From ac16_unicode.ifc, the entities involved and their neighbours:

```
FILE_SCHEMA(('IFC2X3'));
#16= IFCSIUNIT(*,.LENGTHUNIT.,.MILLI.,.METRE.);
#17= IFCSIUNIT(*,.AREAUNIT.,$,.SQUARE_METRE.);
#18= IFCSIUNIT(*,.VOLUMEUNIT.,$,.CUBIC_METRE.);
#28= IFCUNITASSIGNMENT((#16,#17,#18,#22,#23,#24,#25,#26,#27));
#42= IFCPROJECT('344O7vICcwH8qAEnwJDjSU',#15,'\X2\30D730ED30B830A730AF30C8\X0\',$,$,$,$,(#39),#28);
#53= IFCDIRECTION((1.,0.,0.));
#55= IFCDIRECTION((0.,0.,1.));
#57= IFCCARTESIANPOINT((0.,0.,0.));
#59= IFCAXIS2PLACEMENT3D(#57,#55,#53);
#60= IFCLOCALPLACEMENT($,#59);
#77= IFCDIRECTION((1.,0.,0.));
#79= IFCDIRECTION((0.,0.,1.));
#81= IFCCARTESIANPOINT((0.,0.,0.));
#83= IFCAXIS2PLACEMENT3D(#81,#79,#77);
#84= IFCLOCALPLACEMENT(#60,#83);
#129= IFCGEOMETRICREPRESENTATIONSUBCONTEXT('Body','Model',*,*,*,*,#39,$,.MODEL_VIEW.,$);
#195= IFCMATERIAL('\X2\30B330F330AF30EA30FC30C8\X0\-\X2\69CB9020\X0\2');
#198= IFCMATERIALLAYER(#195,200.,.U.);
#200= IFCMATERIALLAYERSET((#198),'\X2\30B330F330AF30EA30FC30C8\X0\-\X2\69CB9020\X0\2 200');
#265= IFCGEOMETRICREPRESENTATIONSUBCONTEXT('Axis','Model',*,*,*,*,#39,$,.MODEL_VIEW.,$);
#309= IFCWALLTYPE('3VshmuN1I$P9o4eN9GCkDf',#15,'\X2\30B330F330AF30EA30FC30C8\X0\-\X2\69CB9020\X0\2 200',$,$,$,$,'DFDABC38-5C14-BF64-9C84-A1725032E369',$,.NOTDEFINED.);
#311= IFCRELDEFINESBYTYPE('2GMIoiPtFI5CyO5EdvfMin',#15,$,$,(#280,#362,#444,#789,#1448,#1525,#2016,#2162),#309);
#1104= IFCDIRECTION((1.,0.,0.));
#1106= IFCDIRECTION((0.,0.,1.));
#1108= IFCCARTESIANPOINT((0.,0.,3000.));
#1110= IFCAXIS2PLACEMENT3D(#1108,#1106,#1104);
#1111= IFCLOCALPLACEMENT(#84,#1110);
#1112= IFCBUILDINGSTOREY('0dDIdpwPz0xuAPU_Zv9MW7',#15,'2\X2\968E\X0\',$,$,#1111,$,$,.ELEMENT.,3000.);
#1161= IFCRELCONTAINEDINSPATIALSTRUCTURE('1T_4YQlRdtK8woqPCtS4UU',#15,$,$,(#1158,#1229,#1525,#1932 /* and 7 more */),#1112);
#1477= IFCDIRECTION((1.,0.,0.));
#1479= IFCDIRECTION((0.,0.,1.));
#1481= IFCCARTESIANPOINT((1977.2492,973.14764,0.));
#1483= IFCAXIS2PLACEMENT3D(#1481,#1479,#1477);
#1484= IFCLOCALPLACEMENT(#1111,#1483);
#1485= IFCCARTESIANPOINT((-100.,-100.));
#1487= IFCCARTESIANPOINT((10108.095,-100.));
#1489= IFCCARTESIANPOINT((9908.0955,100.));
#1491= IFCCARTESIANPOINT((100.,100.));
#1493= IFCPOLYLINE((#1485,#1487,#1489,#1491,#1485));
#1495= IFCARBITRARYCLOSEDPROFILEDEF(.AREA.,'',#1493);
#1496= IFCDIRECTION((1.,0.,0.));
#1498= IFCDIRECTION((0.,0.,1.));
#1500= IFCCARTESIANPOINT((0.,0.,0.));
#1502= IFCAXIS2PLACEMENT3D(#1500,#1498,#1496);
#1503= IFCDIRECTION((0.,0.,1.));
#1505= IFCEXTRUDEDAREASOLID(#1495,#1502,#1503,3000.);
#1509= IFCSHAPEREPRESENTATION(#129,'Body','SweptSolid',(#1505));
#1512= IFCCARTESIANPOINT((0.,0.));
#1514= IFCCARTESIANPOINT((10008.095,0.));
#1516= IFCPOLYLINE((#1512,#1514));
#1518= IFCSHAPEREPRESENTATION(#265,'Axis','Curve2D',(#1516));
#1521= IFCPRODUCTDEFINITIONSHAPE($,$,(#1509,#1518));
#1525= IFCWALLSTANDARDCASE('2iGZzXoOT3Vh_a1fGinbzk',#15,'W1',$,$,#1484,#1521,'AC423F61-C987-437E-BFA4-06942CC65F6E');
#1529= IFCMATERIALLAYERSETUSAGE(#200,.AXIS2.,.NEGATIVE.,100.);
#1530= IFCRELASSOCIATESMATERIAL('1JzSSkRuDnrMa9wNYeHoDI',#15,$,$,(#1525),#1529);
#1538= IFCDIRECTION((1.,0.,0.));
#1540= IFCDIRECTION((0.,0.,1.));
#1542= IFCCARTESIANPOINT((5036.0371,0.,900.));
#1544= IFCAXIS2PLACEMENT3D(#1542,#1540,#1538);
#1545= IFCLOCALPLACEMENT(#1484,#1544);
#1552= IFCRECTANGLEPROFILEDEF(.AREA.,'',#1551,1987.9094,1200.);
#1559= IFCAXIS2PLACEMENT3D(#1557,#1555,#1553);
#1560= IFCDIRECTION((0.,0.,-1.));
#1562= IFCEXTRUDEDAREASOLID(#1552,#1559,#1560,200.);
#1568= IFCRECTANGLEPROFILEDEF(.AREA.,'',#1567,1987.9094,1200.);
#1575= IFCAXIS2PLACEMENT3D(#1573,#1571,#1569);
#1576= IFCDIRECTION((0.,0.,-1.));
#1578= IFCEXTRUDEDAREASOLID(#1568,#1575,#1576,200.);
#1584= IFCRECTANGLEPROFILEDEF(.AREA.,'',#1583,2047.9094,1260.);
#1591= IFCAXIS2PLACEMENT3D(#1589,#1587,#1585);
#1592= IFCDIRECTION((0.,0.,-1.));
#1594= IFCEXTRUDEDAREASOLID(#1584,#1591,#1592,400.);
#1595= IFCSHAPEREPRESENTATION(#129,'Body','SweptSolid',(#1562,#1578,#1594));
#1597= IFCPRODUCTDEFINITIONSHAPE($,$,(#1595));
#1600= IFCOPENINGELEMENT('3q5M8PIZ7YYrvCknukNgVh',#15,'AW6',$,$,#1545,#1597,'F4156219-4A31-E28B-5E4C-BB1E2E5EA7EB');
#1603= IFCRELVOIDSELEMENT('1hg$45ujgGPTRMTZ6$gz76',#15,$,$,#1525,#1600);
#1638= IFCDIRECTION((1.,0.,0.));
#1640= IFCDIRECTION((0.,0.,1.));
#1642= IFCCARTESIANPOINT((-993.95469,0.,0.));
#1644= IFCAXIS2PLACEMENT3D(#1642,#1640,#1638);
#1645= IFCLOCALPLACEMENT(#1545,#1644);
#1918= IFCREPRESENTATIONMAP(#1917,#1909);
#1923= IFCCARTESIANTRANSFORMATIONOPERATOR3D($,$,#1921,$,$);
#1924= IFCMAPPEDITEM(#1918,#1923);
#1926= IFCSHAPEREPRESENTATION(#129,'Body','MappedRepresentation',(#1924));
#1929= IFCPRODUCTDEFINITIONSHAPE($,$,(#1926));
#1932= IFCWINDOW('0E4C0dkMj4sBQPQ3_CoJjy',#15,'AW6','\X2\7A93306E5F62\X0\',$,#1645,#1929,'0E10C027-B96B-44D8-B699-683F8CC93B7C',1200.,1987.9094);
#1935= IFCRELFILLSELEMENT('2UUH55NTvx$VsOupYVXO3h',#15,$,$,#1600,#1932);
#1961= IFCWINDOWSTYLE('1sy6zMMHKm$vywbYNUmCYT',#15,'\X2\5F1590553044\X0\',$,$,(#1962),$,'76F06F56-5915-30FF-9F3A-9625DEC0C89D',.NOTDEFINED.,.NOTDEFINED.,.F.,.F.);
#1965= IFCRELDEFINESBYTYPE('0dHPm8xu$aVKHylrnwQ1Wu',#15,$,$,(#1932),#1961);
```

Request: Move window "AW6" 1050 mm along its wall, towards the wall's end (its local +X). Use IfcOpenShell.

```python
import ifcopenshell
import ifcopenshell.api.geometry
import ifcopenshell.util.placement

model = ifcopenshell.open("ac16_unicode.ifc")

window = model.by_guid("0E4C0dkMj4sBQPQ3_CoJjy")
opening = window.FillsVoids[0].RelatingOpeningElement
wall = opening.VoidsElements[0].RelatingBuildingElement

wall_matrix = ifcopenshell.util.placement.get_local_placement(wall.ObjectPlacement)
shift = wall_matrix[:3, 0] * 1050.0
before = ifcopenshell.util.placement.get_local_placement(window.ObjectPlacement)[:3, 3].copy()

# The window is placed relative to its opening, so it follows when the opening moves.
matrix = ifcopenshell.util.placement.get_local_placement(opening.ObjectPlacement)
matrix[:3, 3] += shift
ifcopenshell.api.geometry.edit_object_placement(
    model, product=opening, matrix=matrix, is_si=False, should_transform_children=True
)

after = ifcopenshell.util.placement.get_local_placement(window.ObjectPlacement)[:3, 3]
print("window moved by", (after - before).round(3) + 0.0)

model.write("ac16_unicode_updated.ifc")
```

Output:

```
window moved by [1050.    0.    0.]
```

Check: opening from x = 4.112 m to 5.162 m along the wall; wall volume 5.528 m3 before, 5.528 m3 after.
